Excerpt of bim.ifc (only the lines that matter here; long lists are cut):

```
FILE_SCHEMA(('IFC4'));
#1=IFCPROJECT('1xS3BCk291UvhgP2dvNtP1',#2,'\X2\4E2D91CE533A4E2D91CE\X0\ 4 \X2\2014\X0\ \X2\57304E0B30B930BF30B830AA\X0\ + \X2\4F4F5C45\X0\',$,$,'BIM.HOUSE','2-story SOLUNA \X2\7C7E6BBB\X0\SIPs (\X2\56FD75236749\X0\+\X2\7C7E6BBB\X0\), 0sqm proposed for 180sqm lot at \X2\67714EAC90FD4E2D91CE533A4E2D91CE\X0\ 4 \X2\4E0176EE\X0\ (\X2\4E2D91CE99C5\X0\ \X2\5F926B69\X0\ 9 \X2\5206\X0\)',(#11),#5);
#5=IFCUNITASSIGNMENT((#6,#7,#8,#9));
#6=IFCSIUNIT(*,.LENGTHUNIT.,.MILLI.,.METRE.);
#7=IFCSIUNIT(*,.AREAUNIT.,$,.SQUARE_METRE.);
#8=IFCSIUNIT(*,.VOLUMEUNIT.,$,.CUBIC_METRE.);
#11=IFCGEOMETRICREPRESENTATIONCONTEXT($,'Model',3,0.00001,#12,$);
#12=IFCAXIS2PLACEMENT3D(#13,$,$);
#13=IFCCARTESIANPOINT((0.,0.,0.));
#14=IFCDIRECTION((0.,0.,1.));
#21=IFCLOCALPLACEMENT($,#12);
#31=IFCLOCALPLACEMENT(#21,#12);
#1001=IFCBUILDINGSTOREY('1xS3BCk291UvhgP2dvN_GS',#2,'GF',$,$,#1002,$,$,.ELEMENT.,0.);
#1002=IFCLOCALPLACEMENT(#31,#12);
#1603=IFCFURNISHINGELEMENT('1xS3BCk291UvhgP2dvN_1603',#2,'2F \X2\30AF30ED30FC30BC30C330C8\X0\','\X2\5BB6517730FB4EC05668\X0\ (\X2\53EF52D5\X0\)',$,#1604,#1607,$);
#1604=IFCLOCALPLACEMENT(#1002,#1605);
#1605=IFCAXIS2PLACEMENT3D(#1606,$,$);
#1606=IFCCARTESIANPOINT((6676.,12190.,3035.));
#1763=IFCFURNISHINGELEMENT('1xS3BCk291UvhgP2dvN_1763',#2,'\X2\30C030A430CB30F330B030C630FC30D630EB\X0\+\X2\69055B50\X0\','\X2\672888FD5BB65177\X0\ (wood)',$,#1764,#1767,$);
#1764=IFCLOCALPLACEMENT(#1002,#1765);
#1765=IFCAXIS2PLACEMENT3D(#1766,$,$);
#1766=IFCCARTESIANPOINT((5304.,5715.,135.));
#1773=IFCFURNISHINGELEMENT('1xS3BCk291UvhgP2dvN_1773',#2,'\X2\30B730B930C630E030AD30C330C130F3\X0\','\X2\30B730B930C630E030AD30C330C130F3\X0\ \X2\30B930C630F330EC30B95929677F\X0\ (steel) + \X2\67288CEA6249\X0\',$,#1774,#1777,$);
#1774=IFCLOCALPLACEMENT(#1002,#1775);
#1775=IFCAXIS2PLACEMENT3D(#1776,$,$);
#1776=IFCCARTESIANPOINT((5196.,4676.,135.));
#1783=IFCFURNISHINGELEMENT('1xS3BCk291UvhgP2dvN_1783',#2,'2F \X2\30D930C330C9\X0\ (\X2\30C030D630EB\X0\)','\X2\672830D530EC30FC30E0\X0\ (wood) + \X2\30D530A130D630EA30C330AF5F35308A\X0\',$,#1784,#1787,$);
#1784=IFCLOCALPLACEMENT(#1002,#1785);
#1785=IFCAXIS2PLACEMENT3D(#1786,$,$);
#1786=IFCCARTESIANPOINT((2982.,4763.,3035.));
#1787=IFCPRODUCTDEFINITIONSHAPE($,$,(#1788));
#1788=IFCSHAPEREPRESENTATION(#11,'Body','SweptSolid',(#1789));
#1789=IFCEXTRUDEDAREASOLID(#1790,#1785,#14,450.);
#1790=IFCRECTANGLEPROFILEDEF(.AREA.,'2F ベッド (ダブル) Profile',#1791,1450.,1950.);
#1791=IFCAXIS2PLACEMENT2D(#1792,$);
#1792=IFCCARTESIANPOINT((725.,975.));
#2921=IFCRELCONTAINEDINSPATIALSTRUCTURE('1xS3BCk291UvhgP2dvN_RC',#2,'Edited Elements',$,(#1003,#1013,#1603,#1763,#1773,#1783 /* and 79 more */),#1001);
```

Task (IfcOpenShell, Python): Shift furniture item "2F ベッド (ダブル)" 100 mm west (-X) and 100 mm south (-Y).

```python
import ifcopenshell
import ifcopenshell.api.geometry
import ifcopenshell.util.placement
import ifcopenshell.util.unit

model = ifcopenshell.open("bim.ifc")
unit_scale = ifcopenshell.util.unit.calculate_unit_scale(model)

item = model.by_guid("1xS3BCk291UvhgP2dvN_1783")
matrix = ifcopenshell.util.placement.get_local_placement(item.ObjectPlacement)
matrix[0, 3] -= 0.1 / unit_scale
matrix[1, 3] -= 0.1 / unit_scale
ifcopenshell.api.geometry.edit_object_placement(model, product=item, matrix=matrix, is_si=False)

print(ifcopenshell.util.placement.get_local_placement(item.ObjectPlacement).round(3) + 0.0)

model.write("bim_edited.ifc")
```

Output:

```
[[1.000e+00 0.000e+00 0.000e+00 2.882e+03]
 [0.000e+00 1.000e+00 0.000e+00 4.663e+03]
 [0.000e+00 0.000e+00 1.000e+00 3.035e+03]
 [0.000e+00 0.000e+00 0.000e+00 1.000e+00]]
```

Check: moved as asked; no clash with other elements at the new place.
